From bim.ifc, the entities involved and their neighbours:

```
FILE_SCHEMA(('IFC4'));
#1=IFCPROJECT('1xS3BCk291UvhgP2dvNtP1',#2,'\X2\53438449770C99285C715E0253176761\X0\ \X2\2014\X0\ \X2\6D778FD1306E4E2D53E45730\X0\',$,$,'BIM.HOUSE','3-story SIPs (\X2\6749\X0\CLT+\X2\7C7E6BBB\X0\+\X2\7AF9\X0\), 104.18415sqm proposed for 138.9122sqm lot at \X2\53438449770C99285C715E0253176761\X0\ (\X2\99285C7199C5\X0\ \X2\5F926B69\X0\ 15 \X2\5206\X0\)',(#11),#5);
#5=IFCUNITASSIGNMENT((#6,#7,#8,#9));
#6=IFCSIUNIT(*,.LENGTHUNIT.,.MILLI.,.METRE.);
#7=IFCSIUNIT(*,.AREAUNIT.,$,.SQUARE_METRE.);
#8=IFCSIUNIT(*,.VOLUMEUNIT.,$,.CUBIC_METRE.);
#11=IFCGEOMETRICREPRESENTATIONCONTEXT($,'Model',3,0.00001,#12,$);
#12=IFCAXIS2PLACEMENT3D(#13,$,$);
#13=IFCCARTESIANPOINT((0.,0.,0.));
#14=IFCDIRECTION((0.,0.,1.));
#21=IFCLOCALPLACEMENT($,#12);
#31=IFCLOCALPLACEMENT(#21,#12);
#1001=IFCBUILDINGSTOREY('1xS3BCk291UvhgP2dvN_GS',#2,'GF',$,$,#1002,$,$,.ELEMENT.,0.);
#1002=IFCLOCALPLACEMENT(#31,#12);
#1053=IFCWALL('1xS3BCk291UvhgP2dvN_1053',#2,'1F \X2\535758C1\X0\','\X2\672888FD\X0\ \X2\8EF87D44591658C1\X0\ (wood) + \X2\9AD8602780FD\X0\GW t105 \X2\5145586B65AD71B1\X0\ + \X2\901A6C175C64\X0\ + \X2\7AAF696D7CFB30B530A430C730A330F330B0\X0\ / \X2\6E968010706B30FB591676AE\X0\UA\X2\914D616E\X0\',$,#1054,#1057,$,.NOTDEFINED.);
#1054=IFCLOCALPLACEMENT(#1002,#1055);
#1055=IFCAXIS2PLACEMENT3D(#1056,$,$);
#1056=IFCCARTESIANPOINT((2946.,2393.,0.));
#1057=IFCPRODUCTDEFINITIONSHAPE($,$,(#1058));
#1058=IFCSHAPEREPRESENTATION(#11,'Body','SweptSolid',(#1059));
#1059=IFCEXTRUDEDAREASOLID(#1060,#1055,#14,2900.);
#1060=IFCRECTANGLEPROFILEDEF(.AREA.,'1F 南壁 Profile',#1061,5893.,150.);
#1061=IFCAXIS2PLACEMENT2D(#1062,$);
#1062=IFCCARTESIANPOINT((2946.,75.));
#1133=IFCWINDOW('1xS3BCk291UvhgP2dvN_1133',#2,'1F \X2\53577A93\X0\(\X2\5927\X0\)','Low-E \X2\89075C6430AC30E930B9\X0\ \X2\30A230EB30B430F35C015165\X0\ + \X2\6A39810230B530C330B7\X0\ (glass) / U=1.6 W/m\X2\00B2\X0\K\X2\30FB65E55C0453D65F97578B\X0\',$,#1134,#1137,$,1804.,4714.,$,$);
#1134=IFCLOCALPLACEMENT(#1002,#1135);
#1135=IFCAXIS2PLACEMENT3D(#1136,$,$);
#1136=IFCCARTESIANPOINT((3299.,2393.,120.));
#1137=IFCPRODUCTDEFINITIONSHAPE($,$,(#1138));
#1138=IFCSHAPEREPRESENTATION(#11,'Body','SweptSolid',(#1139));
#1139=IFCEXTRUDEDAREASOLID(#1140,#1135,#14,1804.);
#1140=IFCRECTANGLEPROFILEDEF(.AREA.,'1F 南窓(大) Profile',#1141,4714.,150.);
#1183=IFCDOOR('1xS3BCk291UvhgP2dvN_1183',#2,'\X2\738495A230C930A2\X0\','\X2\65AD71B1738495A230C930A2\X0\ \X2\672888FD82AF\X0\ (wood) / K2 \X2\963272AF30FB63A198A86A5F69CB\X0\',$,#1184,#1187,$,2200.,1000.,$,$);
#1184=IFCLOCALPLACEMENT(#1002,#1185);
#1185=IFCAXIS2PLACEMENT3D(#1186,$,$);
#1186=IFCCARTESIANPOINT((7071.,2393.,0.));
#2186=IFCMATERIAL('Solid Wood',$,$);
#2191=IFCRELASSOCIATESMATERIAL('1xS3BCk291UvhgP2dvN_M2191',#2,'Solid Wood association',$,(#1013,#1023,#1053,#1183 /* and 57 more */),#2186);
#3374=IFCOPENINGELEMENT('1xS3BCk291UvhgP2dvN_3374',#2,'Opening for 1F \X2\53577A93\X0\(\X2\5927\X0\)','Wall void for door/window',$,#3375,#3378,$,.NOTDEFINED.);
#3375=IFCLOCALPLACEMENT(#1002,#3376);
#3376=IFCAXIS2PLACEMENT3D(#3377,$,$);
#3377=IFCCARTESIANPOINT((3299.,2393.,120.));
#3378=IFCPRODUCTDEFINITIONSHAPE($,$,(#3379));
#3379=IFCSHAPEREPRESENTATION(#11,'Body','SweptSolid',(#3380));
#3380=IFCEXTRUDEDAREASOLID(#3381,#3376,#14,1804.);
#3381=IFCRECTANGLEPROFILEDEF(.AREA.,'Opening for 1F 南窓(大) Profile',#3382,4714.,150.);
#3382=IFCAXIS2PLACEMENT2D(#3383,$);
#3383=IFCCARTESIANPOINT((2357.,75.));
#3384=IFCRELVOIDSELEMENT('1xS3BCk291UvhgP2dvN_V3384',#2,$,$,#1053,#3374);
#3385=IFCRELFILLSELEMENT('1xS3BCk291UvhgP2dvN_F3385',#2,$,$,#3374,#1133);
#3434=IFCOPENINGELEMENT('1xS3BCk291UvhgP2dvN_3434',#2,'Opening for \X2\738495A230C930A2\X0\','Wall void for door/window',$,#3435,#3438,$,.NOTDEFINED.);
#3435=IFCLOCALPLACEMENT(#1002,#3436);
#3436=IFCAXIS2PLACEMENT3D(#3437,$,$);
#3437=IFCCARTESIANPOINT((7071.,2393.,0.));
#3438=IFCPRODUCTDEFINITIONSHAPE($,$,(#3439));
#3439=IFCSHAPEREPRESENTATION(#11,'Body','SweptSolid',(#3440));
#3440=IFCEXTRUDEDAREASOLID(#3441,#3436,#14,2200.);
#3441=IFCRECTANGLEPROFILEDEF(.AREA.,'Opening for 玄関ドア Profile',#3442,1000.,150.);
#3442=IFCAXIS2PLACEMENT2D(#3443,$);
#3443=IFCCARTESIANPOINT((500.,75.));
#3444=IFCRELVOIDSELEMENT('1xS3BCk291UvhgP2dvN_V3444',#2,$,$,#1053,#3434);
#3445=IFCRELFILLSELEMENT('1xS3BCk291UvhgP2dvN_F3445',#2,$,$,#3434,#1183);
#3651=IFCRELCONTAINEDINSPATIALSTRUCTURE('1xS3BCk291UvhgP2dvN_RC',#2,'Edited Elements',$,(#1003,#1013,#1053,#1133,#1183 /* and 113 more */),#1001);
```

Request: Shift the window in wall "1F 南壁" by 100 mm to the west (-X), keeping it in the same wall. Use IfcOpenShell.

```python
import ifcopenshell
import ifcopenshell.api.geometry
import ifcopenshell.util.placement
import ifcopenshell.util.unit

model = ifcopenshell.open("bim.ifc")
unit_scale = ifcopenshell.util.unit.calculate_unit_scale(model)

window = model.by_id(1133)
opening = window.FillsVoids[0].RelatingOpeningElement
wall = opening.VoidsElements[0].RelatingBuildingElement

wall_matrix = ifcopenshell.util.placement.get_local_placement(wall.ObjectPlacement)
shift = wall_matrix[:3, 0] * -0.1 / unit_scale
before = ifcopenshell.util.placement.get_local_placement(window.ObjectPlacement)[:3, 3].copy()

# The window is not placed relative to its opening, so move both.
for product in (opening, window):
    matrix = ifcopenshell.util.placement.get_local_placement(product.ObjectPlacement)
    matrix[:3, 3] += shift
    ifcopenshell.api.geometry.edit_object_placement(model, product=product, matrix=matrix, is_si=False)

after = ifcopenshell.util.placement.get_local_placement(window.ObjectPlacement)[:3, 3]
print("window moved by", (after - before).round(3) + 0.0)

model.write("bim_edited.ifc")
```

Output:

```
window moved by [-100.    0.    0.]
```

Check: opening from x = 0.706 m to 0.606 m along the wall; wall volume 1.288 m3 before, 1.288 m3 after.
